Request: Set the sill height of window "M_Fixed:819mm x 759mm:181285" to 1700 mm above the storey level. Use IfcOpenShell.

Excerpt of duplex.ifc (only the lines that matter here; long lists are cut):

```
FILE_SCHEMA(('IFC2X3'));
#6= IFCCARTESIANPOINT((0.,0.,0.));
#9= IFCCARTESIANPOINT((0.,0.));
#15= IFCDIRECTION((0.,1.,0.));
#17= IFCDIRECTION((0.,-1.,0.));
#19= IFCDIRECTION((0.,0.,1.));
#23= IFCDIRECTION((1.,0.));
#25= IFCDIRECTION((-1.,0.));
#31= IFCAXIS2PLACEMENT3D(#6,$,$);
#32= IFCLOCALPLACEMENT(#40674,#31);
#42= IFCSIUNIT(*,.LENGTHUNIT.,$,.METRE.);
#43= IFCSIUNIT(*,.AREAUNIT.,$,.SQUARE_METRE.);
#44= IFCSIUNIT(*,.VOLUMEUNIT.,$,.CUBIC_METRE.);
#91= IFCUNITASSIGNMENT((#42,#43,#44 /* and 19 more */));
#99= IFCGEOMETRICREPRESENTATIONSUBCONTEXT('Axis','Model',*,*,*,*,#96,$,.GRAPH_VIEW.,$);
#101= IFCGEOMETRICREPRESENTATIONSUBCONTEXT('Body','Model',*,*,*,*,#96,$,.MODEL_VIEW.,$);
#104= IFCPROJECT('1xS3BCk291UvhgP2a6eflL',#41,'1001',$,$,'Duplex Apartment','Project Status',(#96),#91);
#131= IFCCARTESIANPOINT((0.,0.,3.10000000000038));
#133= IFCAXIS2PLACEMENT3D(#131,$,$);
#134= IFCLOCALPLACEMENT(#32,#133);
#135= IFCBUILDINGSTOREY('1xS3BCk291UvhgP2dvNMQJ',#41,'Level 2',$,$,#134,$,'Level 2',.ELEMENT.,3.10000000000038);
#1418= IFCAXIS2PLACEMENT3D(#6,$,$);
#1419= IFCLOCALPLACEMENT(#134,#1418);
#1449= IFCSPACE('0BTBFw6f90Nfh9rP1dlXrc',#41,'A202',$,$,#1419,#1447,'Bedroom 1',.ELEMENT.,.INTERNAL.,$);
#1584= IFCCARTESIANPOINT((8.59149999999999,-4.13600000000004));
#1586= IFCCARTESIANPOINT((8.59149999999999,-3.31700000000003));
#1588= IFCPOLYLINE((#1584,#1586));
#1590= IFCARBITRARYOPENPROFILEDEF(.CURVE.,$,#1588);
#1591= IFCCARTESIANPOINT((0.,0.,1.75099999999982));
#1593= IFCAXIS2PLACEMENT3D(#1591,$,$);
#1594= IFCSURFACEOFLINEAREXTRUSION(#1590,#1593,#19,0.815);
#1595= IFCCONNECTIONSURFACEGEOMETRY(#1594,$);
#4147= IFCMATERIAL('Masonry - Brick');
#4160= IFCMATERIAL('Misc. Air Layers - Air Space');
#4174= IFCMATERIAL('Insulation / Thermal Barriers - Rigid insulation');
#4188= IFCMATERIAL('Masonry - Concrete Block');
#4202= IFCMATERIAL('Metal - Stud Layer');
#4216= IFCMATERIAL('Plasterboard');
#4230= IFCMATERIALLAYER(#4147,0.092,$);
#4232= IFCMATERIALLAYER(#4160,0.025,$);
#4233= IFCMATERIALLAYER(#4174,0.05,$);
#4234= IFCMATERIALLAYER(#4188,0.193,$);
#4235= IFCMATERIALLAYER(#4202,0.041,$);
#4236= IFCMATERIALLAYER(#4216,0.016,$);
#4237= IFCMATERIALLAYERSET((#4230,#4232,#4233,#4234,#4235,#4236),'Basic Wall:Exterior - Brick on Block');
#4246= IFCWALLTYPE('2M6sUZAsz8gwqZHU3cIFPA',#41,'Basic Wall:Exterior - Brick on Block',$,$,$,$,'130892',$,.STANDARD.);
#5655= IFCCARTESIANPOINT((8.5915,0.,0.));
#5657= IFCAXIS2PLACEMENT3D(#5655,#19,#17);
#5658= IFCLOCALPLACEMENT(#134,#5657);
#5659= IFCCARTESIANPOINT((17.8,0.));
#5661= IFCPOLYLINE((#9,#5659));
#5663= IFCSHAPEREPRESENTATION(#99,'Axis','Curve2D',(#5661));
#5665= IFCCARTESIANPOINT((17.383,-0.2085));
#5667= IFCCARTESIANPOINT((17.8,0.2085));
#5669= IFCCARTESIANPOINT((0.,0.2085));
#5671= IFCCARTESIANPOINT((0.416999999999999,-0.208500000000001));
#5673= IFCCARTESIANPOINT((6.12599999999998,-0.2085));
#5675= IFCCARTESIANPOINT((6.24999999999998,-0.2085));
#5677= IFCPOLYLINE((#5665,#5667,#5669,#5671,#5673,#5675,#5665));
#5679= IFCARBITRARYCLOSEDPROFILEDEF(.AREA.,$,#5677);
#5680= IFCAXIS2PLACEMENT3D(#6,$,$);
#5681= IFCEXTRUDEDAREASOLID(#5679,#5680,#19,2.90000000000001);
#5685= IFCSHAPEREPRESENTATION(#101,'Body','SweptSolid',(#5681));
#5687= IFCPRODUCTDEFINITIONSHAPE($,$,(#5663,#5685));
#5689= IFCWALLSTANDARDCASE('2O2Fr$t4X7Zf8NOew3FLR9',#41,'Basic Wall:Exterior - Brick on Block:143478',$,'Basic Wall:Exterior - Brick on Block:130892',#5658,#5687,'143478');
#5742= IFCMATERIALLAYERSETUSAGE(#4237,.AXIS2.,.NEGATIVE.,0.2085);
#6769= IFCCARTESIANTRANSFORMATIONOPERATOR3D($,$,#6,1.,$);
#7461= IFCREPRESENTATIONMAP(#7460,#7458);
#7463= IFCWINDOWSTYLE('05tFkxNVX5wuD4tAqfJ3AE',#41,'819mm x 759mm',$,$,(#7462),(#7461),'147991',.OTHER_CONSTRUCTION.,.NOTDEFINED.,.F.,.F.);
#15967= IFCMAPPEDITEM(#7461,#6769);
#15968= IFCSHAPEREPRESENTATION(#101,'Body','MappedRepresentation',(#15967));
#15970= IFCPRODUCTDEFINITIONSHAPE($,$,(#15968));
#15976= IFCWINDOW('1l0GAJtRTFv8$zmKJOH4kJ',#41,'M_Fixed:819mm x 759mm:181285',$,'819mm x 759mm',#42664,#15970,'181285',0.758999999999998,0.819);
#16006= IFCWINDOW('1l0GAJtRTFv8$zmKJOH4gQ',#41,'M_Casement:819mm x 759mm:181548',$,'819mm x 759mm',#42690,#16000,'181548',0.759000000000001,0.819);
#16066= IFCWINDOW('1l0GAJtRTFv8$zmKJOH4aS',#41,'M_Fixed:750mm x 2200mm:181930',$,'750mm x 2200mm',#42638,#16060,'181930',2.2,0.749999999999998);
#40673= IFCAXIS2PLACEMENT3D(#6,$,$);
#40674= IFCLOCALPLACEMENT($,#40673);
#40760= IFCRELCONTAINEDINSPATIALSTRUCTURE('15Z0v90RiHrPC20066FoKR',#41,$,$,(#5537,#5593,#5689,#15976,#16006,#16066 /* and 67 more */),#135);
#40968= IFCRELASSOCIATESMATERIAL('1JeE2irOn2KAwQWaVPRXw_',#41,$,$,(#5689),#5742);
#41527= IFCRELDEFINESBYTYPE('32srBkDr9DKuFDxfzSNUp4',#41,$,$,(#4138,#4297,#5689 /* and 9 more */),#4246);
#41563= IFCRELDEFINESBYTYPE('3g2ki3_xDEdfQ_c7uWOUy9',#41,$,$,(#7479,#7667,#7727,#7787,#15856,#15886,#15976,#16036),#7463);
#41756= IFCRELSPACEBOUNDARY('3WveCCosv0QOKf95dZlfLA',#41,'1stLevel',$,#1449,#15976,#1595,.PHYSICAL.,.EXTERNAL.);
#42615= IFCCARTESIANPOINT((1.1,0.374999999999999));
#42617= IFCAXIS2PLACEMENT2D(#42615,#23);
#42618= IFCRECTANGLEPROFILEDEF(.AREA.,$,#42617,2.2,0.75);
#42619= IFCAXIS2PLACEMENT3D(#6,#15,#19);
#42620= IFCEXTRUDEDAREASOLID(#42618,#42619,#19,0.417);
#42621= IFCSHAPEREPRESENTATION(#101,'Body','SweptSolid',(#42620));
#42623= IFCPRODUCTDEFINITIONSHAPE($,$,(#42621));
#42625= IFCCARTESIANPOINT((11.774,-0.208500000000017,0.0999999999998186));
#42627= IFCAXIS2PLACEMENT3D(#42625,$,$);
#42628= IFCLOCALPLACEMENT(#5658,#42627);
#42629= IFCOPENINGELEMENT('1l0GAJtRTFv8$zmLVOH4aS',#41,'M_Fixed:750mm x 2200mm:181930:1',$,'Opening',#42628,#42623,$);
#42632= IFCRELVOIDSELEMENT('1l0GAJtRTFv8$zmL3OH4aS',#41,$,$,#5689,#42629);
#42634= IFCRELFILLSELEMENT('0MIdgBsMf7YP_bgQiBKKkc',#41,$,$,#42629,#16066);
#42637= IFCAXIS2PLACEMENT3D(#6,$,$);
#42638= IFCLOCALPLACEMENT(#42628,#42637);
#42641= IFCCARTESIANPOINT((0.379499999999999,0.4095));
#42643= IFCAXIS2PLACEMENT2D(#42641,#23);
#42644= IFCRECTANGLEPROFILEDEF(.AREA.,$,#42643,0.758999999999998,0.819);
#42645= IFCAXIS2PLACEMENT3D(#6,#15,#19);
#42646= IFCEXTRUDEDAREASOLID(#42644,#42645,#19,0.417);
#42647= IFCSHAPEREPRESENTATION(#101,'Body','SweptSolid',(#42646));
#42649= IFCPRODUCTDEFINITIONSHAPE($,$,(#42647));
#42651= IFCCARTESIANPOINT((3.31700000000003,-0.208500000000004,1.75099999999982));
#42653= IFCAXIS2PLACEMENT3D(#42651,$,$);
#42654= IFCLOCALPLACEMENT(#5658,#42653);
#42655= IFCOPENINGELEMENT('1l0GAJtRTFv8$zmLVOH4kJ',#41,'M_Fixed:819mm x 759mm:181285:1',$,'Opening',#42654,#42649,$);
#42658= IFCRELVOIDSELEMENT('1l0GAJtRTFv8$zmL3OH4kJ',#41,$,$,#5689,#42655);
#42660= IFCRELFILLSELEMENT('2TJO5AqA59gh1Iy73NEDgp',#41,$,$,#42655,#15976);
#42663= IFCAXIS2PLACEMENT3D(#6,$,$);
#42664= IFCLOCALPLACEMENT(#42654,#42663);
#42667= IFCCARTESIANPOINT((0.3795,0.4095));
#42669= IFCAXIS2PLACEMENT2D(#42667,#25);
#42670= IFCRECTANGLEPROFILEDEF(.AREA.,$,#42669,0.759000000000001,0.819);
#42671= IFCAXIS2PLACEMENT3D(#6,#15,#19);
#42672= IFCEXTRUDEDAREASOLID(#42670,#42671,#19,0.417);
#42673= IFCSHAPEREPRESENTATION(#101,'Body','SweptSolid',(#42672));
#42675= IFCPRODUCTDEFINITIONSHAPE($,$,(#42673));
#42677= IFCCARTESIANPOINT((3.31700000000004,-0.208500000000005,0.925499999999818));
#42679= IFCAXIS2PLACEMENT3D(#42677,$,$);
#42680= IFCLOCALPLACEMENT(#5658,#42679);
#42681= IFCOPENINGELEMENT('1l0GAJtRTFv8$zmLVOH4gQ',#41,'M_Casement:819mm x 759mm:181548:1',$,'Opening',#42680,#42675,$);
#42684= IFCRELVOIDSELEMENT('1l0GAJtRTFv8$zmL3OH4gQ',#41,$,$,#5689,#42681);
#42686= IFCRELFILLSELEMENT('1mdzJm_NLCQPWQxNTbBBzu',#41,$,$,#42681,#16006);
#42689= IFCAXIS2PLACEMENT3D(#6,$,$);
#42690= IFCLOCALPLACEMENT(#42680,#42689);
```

```python
import numpy as np
import ifcopenshell
import ifcopenshell.api.geometry
import ifcopenshell.geom
import ifcopenshell.util.element
import ifcopenshell.util.placement
import ifcopenshell.util.shape
import ifcopenshell.util.unit

model = ifcopenshell.open("duplex.ifc")
unit_scale = ifcopenshell.util.unit.calculate_unit_scale(model)

window = model.by_guid("1l0GAJtRTFv8$zmKJOH4kJ")
opening = window.FillsVoids[0].RelatingOpeningElement
storey = ifcopenshell.util.element.get_container(window, ifc_class="IfcBuildingStorey")
level = ifcopenshell.util.placement.get_local_placement(storey.ObjectPlacement)[2, 3]

# The opening's origin need not be at the sill, so measure its lowest point.
shape = ifcopenshell.geom.create_shape(ifcopenshell.geom.settings(), opening)
bottom = ifcopenshell.util.shape.get_shape_bottom_elevation(shape, shape.geometry) / unit_scale
dz = level + 1.7 - bottom

shift = np.array([0.0, 0.0, dz])
# The window is placed relative to its opening, so it follows when the opening moves.
matrix = ifcopenshell.util.placement.get_local_placement(opening.ObjectPlacement)
matrix[:3, 3] += shift
ifcopenshell.api.geometry.edit_object_placement(
    model, product=opening, matrix=matrix, is_si=False, should_transform_children=True
)

# Space boundary surfaces are stored in each space's coordinates; move them too.
for rel in window.ProvidesBoundaries:
    if not rel.ConnectionGeometry:
        continue
    surface = rel.ConnectionGeometry.SurfaceOnRelatingElement
    space_matrix = ifcopenshell.util.placement.get_local_placement(rel.RelatingSpace.ObjectPlacement)
    point = np.array(surface.Position.Location.Coordinates) + space_matrix[:3, :3].T @ shift
    surface.Position = model.createIfcAxis2Placement3D(
        model.createIfcCartesianPoint(point.tolist()), surface.Position.Axis, surface.Position.RefDirection
    )

print(f"moved by {dz * unit_scale:+.3f} m")

model.write("duplex_updated.ifc")
```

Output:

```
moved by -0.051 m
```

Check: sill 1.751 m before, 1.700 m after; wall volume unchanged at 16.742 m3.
